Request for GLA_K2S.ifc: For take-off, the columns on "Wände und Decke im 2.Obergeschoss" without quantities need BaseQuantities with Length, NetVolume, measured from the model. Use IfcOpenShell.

First a look at what the model holds.

```python
import ifcopenshell
import ifcopenshell.util.element
import ifcopenshell.util.unit

model = ifcopenshell.open("GLA_K2S.ifc")
print(model.schema)
for unit_type in ("LENGTHUNIT", "AREAUNIT", "VOLUMEUNIT"):
    print(unit_type, ifcopenshell.util.unit.calculate_unit_scale(model, unit_type))
storey = next(s for s in model.by_type("IfcBuildingStorey") if s.Name == "Wände und Decke im 2.Obergeschoss")
columns = [e for e in ifcopenshell.util.element.get_decomposition(storey) if e.is_a("IfcColumn")]
for e in sorted(columns, key=lambda e: e.id()):
    print(e.id(), e.is_a(), e.Name, list(ifcopenshell.util.element.get_psets(e, qtos_only=True)), sep=" | ")
```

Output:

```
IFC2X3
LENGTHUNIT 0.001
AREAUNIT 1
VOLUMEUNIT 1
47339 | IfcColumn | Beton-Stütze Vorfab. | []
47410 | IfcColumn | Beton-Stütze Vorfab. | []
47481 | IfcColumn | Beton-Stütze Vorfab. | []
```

```python
import ifcopenshell
import ifcopenshell.api.pset
import ifcopenshell.geom
import ifcopenshell.util.element
import ifcopenshell.util.shape
import ifcopenshell.util.unit

model = ifcopenshell.open("GLA_K2S.ifc")
unit_scale = ifcopenshell.util.unit.calculate_unit_scale(model)
volume_scale = ifcopenshell.util.unit.calculate_unit_scale(model, "VOLUMEUNIT")
settings = ifcopenshell.geom.settings()

storey = next(s for s in model.by_type("IfcBuildingStorey") if s.Name == "Wände und Decke im 2.Obergeschoss")
columns = [e for e in ifcopenshell.util.element.get_decomposition(storey) if e.is_a("IfcColumn")]

for e in sorted(columns, key=lambda e: e.id()):
    if ifcopenshell.util.element.get_psets(e, qtos_only=True, should_inherit=False):
        continue
    # Geometry comes back in metres, in the element's own axes.
    shape = ifcopenshell.geom.create_shape(settings, e)
    values = {
        "Length": ifcopenshell.util.shape.get_z(shape.geometry) / unit_scale,
        "NetVolume": ifcopenshell.util.shape.get_volume(shape.geometry) / volume_scale,
    }
    qto = ifcopenshell.api.pset.add_qto(model, product=e, name="BaseQuantities")
    ifcopenshell.api.pset.edit_qto(model, qto=qto, properties=values)
    print(e.id(), {k: round(v, 3) for k, v in values.items()})

model.write("GLA_K2S_updated.ifc")
```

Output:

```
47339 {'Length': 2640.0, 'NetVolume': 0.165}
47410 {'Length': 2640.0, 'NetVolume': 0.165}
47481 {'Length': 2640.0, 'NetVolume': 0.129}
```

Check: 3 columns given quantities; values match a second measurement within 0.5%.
